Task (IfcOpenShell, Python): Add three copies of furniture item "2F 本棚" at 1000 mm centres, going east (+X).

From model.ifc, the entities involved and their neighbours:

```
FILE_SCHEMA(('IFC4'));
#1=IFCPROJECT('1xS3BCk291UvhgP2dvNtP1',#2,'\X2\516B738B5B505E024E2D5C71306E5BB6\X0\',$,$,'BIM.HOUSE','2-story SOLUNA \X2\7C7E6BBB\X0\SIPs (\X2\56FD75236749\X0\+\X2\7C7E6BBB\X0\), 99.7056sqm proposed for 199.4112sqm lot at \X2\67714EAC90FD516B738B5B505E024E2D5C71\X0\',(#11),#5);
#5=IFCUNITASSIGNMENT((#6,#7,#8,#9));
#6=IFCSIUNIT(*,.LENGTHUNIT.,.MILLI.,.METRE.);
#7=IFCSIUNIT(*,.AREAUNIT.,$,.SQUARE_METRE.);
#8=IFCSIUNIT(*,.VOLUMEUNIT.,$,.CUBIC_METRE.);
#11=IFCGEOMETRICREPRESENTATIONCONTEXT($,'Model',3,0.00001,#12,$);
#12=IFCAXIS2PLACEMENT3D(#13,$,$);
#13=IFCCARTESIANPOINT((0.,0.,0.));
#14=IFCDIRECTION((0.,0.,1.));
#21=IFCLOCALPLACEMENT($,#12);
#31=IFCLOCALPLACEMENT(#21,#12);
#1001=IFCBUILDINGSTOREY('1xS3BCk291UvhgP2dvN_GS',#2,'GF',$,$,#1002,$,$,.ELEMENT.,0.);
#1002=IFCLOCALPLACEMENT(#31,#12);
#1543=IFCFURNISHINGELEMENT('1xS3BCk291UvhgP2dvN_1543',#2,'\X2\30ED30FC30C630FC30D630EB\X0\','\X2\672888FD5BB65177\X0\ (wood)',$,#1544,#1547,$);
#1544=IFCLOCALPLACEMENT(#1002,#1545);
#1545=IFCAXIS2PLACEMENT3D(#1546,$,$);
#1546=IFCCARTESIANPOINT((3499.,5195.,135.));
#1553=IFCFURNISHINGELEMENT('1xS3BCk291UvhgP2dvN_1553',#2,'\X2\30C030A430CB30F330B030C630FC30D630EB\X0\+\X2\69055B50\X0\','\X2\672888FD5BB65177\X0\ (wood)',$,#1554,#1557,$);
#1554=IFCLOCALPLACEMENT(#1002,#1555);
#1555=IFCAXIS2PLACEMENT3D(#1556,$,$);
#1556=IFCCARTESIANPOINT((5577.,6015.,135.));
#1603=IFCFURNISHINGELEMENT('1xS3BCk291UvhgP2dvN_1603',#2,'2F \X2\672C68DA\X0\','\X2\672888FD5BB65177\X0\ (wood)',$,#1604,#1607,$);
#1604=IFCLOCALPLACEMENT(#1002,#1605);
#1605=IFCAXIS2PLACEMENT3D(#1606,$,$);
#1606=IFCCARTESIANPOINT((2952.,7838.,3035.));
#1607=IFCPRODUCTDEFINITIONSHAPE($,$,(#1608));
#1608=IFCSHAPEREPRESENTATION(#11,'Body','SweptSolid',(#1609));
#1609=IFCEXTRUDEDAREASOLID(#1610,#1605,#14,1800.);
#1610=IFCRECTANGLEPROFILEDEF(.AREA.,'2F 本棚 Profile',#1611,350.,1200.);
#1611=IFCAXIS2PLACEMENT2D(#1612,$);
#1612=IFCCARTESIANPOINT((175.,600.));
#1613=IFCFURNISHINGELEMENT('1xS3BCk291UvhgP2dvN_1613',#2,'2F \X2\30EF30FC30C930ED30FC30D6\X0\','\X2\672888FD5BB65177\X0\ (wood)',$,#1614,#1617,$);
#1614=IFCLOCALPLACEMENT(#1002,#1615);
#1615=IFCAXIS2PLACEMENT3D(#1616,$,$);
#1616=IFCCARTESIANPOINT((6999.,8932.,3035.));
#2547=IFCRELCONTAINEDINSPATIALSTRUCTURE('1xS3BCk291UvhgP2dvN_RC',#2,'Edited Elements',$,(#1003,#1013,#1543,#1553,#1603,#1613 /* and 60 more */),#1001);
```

```python
import numpy as np
import ifcopenshell
import ifcopenshell.api.geometry
import ifcopenshell.api.root
import ifcopenshell.util.element
import ifcopenshell.util.placement
import ifcopenshell.util.unit

model = ifcopenshell.open("model.ifc")
unit_scale = ifcopenshell.util.unit.calculate_unit_scale(model)


def reuse_history(source, copy):
    """copy_class also copies each property set's owner history, people and application; keep the originals."""
    for rel in copy.IsDefinedBy:
        if rel.is_a("IfcRelDefinesByProperties") and (history := rel.RelatingPropertyDefinition.OwnerHistory):
            rel.RelatingPropertyDefinition.OwnerHistory = source.OwnerHistory
            ifcopenshell.util.element.remove_deep2(model, history)


source = model.by_id(1603)
base = ifcopenshell.util.placement.get_local_placement(source.ObjectPlacement)
step = np.array([1.0, 0.0, 0.0]) * 1 / unit_scale

for i in range(1, 4):
    copy = ifcopenshell.api.root.copy_class(model, product=source)
    copy.Representation = ifcopenshell.util.element.copy_deep(
        model, source.Representation, exclude=["IfcGeometricRepresentationContext", "IfcRepresentationMap"]
    )
    reuse_history(source, copy)
    matrix = base.copy()
    matrix[:3, 3] += i * step
    print("added at", matrix[:3, 3].round(3) + 0.0)
    ifcopenshell.api.geometry.edit_object_placement(model, product=copy, matrix=matrix, is_si=False)

model.write("model-out.ifc")
```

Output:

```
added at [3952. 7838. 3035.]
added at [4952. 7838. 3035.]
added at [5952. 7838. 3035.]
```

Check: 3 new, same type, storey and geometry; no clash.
